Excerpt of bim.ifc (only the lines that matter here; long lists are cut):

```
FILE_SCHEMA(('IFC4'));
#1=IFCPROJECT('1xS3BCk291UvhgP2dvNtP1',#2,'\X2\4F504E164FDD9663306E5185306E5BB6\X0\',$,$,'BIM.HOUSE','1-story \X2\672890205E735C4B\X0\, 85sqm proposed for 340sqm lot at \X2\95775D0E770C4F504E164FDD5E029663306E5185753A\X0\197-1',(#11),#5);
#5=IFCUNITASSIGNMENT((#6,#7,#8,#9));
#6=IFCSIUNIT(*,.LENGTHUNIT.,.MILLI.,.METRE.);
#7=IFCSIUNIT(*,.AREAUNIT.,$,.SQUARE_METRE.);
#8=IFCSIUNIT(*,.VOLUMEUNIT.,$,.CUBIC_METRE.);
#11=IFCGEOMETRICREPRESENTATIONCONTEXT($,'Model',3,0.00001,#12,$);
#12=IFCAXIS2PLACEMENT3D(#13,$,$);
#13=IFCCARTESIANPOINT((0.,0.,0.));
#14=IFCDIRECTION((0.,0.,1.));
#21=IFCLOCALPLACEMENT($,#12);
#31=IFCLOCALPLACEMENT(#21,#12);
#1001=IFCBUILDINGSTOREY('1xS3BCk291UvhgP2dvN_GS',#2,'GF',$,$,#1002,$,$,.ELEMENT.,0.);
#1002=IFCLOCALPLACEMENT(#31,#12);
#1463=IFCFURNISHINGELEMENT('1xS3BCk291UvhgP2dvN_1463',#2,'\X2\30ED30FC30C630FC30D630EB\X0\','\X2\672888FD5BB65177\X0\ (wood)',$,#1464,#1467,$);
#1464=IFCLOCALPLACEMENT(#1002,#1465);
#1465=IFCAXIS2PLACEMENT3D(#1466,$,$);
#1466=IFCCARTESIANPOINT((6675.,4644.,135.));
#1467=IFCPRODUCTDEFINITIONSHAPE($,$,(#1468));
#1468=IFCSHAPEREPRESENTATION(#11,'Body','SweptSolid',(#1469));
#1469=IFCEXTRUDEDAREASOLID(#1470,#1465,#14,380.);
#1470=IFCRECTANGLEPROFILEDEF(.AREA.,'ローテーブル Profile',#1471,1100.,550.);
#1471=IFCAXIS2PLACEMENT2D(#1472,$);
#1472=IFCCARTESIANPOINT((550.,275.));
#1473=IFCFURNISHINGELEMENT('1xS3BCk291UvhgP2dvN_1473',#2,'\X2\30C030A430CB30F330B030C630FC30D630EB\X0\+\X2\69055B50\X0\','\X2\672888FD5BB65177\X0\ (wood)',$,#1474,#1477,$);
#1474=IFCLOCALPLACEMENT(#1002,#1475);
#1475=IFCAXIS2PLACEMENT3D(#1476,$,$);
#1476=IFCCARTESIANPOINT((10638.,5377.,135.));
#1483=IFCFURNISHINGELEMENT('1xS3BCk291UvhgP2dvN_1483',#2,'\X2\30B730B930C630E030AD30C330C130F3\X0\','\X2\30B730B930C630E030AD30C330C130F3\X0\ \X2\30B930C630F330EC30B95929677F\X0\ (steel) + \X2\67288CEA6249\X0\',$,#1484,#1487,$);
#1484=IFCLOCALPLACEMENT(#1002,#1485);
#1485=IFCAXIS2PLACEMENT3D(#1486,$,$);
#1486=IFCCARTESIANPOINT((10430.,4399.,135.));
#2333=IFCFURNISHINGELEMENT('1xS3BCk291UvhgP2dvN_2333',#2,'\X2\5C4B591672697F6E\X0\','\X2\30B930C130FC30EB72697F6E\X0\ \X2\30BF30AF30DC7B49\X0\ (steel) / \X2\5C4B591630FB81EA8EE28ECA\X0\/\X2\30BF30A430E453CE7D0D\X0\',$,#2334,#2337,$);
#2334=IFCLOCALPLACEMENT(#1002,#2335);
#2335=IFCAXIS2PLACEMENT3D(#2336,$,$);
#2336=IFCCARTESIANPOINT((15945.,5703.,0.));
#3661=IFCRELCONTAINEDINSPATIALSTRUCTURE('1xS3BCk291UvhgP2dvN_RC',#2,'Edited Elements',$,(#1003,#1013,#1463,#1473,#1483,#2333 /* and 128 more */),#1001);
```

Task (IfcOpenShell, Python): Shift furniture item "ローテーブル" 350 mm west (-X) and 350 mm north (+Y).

```python
import ifcopenshell
import ifcopenshell.api.geometry
import ifcopenshell.util.placement

model = ifcopenshell.open("bim.ifc")

item = model.by_guid("1xS3BCk291UvhgP2dvN_1463")
matrix = ifcopenshell.util.placement.get_local_placement(item.ObjectPlacement)
matrix[0, 3] -= 350.0
matrix[1, 3] += 350.0
ifcopenshell.api.geometry.edit_object_placement(model, product=item, matrix=matrix, is_si=False)

print(ifcopenshell.util.placement.get_local_placement(item.ObjectPlacement).round(3) + 0.0)

model.write("bim-out.ifc")
```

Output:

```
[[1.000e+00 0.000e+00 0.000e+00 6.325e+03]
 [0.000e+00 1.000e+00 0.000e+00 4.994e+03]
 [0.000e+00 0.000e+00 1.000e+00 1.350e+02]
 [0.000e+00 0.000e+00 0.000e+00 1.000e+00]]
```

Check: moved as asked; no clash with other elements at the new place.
